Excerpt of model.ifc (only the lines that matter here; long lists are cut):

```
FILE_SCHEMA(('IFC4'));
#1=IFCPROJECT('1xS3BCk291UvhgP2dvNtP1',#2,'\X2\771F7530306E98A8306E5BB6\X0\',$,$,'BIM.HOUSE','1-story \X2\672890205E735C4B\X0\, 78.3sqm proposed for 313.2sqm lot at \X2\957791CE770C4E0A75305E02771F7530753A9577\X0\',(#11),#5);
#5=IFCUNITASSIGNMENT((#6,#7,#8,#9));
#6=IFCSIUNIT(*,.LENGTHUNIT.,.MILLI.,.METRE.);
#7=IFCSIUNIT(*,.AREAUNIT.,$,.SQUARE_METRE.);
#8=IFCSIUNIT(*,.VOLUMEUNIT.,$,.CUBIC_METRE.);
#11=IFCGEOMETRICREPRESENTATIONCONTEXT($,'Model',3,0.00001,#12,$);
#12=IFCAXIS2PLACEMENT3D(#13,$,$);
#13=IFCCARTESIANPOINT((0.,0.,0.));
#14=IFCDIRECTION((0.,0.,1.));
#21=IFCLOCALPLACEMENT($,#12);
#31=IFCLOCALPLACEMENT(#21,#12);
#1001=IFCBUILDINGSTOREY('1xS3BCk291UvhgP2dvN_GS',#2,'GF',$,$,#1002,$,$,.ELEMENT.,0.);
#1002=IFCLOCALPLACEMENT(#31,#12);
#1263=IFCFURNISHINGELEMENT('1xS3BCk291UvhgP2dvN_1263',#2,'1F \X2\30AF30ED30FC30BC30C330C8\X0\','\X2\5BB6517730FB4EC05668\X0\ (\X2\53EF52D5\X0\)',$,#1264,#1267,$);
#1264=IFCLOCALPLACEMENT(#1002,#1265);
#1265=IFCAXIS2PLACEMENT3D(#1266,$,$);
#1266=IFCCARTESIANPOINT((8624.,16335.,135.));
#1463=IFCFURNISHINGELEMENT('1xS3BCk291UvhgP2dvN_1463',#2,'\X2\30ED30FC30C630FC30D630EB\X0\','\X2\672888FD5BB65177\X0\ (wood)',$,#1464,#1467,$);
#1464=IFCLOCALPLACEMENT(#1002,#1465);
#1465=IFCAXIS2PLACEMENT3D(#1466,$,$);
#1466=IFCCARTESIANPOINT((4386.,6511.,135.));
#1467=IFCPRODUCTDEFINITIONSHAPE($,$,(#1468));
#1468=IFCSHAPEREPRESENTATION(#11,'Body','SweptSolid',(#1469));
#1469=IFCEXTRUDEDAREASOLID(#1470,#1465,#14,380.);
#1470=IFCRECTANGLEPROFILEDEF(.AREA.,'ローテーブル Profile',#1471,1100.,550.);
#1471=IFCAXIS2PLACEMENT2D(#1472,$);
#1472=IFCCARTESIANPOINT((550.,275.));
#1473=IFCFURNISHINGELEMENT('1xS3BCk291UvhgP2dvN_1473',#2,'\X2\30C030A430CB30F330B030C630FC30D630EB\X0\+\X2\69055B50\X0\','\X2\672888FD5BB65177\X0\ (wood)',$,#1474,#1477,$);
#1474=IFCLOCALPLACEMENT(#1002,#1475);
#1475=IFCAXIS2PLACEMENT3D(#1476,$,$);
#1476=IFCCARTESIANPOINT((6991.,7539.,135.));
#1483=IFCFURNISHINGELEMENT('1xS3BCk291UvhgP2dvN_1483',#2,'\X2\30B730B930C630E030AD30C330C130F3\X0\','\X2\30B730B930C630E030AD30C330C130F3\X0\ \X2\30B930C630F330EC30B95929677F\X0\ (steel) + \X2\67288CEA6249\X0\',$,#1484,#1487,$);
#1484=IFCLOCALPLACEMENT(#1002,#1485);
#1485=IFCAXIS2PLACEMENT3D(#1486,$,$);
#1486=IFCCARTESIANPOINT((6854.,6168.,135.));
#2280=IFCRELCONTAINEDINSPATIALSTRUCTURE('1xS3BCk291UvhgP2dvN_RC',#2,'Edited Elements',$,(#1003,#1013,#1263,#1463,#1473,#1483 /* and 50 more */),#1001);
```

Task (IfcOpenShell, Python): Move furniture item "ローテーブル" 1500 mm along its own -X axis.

```python
import ifcopenshell
import ifcopenshell.api.geometry
import ifcopenshell.util.placement

model = ifcopenshell.open("model.ifc")

item = model.by_id(1463)
matrix = ifcopenshell.util.placement.get_local_placement(item.ObjectPlacement)
matrix[:3, 3] -= matrix[:3, 0] * 1500.0
ifcopenshell.api.geometry.edit_object_placement(model, product=item, matrix=matrix, is_si=False)

print(ifcopenshell.util.placement.get_local_placement(item.ObjectPlacement).round(3) + 0.0)

model.write("model_rev.ifc")
```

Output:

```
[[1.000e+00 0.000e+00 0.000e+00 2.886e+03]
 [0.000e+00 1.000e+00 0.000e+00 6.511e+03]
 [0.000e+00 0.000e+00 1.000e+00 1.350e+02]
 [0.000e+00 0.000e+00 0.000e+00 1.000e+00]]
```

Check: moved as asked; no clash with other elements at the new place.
